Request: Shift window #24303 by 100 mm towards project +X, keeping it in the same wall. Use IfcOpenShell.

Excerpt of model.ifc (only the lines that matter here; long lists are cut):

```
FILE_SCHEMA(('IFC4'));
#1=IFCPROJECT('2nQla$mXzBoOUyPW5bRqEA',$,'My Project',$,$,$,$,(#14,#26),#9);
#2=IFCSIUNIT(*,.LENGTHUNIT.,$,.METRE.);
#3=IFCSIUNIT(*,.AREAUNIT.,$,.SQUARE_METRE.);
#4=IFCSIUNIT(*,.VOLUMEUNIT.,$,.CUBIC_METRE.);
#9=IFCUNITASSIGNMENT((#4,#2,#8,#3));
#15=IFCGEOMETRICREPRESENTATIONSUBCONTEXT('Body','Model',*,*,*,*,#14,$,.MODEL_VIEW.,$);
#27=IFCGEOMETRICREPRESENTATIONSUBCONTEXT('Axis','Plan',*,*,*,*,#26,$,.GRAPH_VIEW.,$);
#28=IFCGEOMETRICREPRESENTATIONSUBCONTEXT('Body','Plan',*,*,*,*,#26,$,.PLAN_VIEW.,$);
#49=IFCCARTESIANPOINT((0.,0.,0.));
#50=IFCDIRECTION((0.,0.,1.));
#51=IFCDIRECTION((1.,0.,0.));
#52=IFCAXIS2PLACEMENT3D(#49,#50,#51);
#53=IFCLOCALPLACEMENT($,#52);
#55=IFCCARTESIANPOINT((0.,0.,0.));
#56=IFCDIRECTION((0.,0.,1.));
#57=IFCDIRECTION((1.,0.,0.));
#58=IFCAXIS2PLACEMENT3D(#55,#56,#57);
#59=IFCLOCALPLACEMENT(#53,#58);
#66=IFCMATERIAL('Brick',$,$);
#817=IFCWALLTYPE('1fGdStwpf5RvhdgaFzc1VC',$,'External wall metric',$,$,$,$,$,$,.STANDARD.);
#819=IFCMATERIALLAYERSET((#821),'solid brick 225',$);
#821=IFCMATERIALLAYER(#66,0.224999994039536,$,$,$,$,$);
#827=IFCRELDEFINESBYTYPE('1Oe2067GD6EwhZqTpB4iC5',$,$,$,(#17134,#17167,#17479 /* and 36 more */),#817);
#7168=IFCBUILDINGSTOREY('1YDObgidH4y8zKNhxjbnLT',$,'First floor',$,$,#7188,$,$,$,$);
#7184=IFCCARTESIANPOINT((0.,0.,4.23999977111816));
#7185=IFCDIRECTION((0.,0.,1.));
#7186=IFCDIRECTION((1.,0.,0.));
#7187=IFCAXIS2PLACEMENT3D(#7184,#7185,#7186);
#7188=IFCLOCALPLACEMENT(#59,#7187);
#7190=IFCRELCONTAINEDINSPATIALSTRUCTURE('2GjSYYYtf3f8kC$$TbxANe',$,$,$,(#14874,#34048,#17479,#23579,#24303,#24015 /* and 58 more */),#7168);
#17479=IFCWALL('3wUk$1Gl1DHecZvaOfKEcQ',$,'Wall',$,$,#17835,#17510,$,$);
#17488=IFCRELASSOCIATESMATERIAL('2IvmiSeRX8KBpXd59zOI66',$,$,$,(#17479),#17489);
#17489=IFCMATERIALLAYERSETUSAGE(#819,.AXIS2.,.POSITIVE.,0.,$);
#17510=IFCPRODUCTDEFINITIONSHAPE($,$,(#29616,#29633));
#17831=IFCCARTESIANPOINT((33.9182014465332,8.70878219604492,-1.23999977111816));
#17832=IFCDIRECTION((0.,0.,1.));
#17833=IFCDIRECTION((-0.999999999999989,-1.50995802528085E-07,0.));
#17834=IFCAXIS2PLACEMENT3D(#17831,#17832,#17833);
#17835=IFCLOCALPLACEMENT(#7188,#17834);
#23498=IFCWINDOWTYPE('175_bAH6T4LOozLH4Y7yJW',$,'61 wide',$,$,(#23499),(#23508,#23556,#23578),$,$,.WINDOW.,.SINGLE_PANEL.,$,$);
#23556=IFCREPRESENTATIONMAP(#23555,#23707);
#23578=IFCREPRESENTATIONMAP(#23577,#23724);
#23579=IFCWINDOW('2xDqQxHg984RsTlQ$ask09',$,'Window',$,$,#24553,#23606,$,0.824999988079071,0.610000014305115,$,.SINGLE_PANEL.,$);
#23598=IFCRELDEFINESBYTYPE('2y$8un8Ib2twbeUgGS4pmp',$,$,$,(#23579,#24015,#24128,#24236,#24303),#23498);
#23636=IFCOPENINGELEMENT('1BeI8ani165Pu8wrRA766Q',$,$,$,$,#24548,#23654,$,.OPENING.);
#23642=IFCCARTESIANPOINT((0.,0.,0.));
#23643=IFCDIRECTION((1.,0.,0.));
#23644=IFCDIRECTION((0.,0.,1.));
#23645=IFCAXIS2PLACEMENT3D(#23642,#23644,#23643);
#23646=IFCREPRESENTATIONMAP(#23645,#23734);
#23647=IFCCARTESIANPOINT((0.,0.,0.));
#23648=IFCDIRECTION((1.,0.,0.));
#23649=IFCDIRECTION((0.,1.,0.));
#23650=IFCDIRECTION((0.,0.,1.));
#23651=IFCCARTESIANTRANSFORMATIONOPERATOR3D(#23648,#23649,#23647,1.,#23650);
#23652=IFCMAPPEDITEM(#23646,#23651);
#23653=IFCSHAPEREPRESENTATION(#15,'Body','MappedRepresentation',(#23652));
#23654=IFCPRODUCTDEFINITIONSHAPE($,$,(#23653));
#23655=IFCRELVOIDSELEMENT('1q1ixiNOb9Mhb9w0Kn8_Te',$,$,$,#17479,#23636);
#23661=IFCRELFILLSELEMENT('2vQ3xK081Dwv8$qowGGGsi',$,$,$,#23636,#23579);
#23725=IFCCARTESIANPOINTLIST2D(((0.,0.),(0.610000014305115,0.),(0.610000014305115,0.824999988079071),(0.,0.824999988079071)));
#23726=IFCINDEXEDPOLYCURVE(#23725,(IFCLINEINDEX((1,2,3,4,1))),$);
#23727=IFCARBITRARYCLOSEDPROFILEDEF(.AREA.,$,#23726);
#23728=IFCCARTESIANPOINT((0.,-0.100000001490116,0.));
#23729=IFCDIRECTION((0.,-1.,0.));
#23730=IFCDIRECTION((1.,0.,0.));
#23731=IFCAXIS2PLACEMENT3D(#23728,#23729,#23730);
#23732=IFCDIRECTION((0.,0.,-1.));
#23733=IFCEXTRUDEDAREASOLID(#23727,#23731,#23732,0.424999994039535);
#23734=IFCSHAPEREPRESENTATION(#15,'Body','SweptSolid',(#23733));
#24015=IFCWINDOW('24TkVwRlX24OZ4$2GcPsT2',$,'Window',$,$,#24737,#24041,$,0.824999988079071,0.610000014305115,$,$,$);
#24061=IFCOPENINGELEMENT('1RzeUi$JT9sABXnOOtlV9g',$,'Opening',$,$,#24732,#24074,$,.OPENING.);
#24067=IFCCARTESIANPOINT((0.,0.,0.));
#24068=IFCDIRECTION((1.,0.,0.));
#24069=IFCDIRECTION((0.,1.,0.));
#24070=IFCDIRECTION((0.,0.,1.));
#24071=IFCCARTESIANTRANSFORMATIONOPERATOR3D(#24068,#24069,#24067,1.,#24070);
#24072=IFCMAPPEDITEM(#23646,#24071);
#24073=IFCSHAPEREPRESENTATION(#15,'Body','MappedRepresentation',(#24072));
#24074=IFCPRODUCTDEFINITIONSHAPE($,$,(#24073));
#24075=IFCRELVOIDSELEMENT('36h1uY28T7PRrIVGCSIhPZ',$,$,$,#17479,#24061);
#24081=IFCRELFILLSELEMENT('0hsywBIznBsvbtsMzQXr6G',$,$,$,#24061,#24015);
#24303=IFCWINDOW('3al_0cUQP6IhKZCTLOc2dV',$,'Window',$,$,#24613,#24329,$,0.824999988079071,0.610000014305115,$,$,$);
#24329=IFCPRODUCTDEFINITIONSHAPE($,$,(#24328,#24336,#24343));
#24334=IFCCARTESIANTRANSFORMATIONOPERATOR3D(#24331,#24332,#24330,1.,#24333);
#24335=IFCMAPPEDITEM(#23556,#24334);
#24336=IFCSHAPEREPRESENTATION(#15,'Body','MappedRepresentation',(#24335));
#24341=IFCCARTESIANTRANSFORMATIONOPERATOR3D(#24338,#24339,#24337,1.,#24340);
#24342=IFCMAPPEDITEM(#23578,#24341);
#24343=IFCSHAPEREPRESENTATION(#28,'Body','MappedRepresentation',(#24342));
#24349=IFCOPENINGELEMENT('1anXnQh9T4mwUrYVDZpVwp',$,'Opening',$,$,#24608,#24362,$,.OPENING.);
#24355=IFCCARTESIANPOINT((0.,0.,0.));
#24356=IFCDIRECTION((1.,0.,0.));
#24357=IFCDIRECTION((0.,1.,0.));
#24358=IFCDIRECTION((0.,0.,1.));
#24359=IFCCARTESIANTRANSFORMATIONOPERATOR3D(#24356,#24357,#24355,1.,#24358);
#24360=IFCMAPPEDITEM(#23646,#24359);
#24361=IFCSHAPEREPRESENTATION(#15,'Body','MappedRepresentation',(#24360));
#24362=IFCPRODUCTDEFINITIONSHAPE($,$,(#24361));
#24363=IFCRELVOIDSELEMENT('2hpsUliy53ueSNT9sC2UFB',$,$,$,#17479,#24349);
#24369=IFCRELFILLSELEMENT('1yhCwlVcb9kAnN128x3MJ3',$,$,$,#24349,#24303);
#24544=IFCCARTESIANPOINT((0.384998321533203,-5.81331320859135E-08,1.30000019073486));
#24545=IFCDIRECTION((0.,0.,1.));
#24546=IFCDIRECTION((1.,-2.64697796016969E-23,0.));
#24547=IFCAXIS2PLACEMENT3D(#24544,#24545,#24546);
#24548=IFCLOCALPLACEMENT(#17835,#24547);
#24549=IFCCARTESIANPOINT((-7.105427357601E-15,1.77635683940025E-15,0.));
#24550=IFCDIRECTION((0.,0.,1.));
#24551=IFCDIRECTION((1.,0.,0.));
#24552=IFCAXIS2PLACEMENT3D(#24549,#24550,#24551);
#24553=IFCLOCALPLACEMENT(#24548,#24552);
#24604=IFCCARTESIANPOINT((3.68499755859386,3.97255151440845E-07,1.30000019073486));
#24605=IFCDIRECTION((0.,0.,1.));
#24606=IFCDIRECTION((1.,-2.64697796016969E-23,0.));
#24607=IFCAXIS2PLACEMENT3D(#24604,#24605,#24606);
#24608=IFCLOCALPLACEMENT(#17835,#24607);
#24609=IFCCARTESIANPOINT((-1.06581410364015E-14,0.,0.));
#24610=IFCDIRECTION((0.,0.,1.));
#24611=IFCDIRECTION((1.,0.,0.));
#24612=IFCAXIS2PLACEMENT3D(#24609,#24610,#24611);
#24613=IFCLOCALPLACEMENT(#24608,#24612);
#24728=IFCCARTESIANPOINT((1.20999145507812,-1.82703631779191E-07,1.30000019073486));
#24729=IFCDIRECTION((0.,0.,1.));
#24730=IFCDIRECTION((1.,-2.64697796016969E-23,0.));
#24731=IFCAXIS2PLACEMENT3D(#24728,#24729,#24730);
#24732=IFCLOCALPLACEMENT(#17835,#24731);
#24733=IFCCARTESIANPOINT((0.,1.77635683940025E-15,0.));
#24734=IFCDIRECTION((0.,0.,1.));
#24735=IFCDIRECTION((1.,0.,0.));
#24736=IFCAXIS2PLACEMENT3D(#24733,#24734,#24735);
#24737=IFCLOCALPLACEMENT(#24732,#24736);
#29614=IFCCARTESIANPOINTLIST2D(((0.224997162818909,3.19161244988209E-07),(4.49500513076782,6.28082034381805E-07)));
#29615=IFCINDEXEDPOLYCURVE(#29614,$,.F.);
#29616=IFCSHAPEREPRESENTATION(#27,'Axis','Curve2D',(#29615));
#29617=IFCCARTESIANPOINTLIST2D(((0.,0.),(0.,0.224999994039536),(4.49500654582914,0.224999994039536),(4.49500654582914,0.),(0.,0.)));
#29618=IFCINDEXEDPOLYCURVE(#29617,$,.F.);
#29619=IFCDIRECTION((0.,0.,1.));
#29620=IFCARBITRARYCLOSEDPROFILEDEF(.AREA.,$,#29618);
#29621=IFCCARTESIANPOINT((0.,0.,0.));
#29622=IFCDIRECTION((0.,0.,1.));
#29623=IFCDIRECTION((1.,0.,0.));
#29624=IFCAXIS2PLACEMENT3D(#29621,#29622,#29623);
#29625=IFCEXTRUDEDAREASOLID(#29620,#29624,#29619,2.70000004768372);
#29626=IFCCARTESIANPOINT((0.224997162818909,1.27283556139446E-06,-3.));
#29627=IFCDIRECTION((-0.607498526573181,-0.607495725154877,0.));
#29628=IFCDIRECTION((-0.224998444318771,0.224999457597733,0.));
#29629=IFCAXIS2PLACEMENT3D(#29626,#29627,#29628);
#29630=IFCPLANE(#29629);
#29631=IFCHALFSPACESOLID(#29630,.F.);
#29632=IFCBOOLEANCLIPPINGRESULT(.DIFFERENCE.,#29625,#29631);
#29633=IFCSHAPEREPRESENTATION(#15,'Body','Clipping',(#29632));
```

```python
import ifcopenshell
import ifcopenshell.api.geometry
import ifcopenshell.util.placement
import ifcopenshell.util.unit

model = ifcopenshell.open("model.ifc")
unit_scale = ifcopenshell.util.unit.calculate_unit_scale(model)

window = model.by_guid("3al_0cUQP6IhKZCTLOc2dV")
opening = window.FillsVoids[0].RelatingOpeningElement
wall = opening.VoidsElements[0].RelatingBuildingElement

wall_matrix = ifcopenshell.util.placement.get_local_placement(wall.ObjectPlacement)
shift = wall_matrix[:3, 0] * -0.1 / unit_scale
before = ifcopenshell.util.placement.get_local_placement(window.ObjectPlacement)[:3, 3].copy()

# The window is placed relative to its opening, so it follows when the opening moves.
matrix = ifcopenshell.util.placement.get_local_placement(opening.ObjectPlacement)
matrix[:3, 3] += shift
ifcopenshell.api.geometry.edit_object_placement(
    model, product=opening, matrix=matrix, is_si=False, should_transform_children=True
)

after = ifcopenshell.util.placement.get_local_placement(window.ObjectPlacement)[:3, 3]
print("window moved by", (after - before).round(3) + 0.0)

model.write("model_rev.ifc")
```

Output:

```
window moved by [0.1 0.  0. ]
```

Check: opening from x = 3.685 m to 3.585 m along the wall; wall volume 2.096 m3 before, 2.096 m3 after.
